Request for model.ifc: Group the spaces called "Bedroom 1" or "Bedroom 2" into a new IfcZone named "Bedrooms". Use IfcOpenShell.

First a look at what the model holds.

```python
import ifcopenshell

model = ifcopenshell.open("model.ifc")
print(model.schema)
seen = {}
for space in model.by_type("IfcSpace"):
    seen[space.LongName] = seen.get(space.LongName, 0) + 1
for name, count in sorted(seen.items(), key=str):
    print(count, "x", name)
print("zones:", [z.Name for z in model.by_type("IfcZone")][:20])
```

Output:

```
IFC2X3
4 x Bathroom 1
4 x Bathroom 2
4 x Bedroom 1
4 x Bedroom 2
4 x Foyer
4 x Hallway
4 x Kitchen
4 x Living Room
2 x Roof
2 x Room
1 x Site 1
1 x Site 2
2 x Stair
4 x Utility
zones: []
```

```python
import ifcopenshell
import ifcopenshell.api.group
import ifcopenshell.api.root

model = ifcopenshell.open("model.ifc")

names = {"Bedroom 1", "Bedroom 2"}
spaces = [s for s in model.by_type("IfcSpace") if s.LongName in names]

zone = ifcopenshell.api.root.create_entity(model, ifc_class="IfcZone", name="Bedrooms")
ifcopenshell.api.group.assign_group(model, products=spaces, group=zone)
print(len(spaces), "spaces in", zone.Name)

model.write("model_updated.ifc")
```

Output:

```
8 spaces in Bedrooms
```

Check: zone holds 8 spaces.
